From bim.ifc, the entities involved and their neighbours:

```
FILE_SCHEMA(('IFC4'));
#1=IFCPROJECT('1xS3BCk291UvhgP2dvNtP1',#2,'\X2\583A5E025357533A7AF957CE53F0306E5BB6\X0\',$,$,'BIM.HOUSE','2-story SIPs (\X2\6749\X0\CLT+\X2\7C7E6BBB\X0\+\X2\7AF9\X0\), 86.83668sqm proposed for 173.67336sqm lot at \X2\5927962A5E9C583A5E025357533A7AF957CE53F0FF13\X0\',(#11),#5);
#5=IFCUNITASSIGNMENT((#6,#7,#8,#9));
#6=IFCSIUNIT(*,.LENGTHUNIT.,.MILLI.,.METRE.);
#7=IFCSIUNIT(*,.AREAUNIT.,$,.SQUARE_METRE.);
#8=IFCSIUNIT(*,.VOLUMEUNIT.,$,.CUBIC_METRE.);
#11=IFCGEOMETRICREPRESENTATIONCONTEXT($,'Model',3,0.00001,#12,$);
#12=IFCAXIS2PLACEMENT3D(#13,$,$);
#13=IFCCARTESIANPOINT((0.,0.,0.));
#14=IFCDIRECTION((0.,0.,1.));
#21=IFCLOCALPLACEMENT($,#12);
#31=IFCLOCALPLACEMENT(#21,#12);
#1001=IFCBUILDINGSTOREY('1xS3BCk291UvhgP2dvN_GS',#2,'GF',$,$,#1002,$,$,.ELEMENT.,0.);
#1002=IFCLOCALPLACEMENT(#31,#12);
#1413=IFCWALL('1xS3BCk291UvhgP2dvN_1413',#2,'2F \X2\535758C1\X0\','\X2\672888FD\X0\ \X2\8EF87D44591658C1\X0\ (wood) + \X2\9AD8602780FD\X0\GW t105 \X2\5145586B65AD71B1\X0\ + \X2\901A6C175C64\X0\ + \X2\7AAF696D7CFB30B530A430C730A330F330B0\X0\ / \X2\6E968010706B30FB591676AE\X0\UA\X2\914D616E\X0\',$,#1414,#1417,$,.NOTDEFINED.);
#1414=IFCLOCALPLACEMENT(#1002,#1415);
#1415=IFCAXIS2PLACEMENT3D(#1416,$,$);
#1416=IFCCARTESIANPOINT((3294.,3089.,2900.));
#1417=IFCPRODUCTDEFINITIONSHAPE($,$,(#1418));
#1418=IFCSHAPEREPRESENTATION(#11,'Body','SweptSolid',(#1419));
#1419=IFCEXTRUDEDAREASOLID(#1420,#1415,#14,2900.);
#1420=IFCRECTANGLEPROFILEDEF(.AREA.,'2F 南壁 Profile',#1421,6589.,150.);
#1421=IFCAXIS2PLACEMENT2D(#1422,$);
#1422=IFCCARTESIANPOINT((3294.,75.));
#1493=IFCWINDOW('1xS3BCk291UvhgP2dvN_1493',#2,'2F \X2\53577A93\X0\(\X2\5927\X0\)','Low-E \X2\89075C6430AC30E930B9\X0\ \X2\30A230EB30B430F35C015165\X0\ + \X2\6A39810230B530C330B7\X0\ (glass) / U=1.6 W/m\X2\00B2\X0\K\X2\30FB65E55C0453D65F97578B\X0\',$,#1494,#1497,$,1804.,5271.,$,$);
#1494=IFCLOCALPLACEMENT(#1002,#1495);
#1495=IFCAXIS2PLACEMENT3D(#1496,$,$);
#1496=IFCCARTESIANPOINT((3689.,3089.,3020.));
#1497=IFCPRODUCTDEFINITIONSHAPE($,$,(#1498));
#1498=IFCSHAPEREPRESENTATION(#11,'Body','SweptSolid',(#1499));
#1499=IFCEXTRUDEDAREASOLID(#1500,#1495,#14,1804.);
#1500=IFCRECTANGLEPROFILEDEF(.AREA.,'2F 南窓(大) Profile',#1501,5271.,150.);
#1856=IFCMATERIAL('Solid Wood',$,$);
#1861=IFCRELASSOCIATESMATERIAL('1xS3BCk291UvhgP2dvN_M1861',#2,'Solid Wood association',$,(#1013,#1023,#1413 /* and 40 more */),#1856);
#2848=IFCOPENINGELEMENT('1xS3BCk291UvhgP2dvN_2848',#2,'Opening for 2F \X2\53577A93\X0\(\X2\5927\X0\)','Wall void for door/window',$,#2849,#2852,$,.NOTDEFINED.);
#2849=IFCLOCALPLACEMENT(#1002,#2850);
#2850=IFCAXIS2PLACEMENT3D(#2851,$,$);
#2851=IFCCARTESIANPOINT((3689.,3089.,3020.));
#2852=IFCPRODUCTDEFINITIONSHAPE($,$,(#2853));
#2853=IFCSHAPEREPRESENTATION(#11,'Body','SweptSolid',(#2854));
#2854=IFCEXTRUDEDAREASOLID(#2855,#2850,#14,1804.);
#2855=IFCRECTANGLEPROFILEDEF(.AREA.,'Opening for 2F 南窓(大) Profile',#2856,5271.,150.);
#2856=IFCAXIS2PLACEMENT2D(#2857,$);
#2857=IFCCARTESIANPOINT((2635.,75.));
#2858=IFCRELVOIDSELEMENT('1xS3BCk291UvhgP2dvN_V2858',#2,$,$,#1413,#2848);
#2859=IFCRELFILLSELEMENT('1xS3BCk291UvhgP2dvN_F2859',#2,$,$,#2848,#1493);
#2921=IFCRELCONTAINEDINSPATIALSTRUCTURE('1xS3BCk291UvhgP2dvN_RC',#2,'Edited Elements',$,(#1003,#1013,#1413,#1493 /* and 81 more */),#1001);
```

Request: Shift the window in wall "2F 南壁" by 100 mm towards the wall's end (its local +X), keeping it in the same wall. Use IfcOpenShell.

```python
import ifcopenshell
import ifcopenshell.api.geometry
import ifcopenshell.util.placement
import ifcopenshell.util.unit

model = ifcopenshell.open("bim.ifc")
unit_scale = ifcopenshell.util.unit.calculate_unit_scale(model)

window = model.by_id(1493)
opening = window.FillsVoids[0].RelatingOpeningElement
wall = opening.VoidsElements[0].RelatingBuildingElement

wall_matrix = ifcopenshell.util.placement.get_local_placement(wall.ObjectPlacement)
shift = wall_matrix[:3, 0] * 0.1 / unit_scale
before = ifcopenshell.util.placement.get_local_placement(window.ObjectPlacement)[:3, 3].copy()

# The window is not placed relative to its opening, so move both.
for product in (opening, window):
    matrix = ifcopenshell.util.placement.get_local_placement(product.ObjectPlacement)
    matrix[:3, 3] += shift
    ifcopenshell.api.geometry.edit_object_placement(model, product=product, matrix=matrix, is_si=False)

after = ifcopenshell.util.placement.get_local_placement(window.ObjectPlacement)[:3, 3]
print("window moved by", (after - before).round(3) + 0.0)

model.write("bim_rev.ifc")
```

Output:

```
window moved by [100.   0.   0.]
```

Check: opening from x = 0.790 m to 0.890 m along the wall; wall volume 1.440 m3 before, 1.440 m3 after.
